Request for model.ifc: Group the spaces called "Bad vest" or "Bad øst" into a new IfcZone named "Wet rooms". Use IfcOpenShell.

First a look at what the model holds.

```python
import ifcopenshell

model = ifcopenshell.open("model.ifc")
print(model.schema)
seen = {}
for space in model.by_type("IfcSpace"):
    seen[space.LongName] = seen.get(space.LongName, 0) + 1
for name, count in sorted(seen.items(), key=str):
    print(count, "x", name)
print("zones:", [z.Name for z in model.by_type("IfcZone")][:20])
```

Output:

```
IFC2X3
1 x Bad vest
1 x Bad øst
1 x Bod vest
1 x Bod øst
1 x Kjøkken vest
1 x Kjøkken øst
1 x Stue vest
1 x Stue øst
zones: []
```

```python
import ifcopenshell
import ifcopenshell.api.group
import ifcopenshell.api.root

model = ifcopenshell.open("model.ifc")

names = {"Bad vest", "Bad øst"}
spaces = [s for s in model.by_type("IfcSpace") if s.LongName in names]

zone = ifcopenshell.api.root.create_entity(model, ifc_class="IfcZone", name="Wet rooms")
ifcopenshell.api.group.assign_group(model, products=spaces, group=zone)
print(len(spaces), "spaces in", zone.Name)

model.write("model_v2.ifc")
```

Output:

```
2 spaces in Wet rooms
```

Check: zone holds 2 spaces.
